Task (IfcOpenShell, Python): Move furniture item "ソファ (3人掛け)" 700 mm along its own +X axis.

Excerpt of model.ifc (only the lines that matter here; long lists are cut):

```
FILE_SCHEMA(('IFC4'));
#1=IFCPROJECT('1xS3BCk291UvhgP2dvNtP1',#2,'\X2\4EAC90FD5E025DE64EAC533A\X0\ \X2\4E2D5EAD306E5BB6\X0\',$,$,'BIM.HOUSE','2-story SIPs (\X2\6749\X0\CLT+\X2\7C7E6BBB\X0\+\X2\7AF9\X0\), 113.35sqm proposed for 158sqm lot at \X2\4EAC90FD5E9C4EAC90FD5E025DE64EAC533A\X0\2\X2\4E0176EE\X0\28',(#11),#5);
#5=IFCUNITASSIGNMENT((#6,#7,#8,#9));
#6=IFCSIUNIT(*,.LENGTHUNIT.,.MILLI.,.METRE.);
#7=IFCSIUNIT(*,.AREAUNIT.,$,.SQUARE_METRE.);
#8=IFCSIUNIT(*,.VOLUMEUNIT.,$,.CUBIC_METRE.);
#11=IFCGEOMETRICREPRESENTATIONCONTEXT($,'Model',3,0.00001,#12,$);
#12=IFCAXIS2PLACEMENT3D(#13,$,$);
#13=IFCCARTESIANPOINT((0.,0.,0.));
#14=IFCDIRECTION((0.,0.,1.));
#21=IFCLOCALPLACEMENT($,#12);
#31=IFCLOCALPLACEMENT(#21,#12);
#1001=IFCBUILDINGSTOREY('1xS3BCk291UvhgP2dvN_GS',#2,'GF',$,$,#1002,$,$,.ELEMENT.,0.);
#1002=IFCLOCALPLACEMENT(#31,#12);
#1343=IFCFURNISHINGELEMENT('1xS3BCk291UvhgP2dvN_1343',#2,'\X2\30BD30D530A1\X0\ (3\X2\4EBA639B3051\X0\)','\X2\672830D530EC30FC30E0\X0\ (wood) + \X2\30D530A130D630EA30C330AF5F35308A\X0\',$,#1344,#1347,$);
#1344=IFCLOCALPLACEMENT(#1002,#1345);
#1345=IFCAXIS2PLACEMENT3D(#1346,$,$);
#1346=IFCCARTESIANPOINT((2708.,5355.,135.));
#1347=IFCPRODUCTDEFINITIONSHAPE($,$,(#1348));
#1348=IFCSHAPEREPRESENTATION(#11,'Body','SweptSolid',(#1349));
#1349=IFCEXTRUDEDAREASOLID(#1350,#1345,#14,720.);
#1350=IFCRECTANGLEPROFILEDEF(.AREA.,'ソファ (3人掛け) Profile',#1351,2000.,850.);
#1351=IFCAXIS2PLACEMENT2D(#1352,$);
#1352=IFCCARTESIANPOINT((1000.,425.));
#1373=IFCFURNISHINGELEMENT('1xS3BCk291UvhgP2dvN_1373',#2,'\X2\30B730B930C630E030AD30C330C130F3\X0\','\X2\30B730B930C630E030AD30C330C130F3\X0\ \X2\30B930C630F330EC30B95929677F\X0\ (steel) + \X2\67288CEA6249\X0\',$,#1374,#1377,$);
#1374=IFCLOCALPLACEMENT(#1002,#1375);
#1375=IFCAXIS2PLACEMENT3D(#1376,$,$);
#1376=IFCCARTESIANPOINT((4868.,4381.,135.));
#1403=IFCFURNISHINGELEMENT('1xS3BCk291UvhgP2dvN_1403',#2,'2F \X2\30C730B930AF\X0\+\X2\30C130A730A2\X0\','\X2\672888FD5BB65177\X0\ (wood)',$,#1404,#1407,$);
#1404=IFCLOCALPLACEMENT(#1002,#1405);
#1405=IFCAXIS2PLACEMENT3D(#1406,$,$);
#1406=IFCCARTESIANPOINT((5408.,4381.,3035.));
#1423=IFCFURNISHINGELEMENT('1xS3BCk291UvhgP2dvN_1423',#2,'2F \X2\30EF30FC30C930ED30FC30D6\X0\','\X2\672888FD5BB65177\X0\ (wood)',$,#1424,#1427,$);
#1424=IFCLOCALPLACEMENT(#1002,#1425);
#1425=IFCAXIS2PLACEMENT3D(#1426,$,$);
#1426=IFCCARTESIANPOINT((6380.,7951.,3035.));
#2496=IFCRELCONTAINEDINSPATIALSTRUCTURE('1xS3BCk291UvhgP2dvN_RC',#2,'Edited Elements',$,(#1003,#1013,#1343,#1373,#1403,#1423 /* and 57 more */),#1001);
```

```python
import ifcopenshell
import ifcopenshell.api.geometry
import ifcopenshell.util.placement

model = ifcopenshell.open("model.ifc")

item = model.by_guid("1xS3BCk291UvhgP2dvN_1343")
matrix = ifcopenshell.util.placement.get_local_placement(item.ObjectPlacement)
matrix[:3, 3] += matrix[:3, 0] * 700.0
ifcopenshell.api.geometry.edit_object_placement(model, product=item, matrix=matrix, is_si=False)

print(ifcopenshell.util.placement.get_local_placement(item.ObjectPlacement).round(3) + 0.0)

model.write("model_edited.ifc")
```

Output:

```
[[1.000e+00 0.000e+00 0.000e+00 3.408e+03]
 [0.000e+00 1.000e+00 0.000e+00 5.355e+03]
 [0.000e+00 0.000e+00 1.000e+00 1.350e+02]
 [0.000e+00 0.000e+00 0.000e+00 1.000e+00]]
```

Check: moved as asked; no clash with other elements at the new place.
